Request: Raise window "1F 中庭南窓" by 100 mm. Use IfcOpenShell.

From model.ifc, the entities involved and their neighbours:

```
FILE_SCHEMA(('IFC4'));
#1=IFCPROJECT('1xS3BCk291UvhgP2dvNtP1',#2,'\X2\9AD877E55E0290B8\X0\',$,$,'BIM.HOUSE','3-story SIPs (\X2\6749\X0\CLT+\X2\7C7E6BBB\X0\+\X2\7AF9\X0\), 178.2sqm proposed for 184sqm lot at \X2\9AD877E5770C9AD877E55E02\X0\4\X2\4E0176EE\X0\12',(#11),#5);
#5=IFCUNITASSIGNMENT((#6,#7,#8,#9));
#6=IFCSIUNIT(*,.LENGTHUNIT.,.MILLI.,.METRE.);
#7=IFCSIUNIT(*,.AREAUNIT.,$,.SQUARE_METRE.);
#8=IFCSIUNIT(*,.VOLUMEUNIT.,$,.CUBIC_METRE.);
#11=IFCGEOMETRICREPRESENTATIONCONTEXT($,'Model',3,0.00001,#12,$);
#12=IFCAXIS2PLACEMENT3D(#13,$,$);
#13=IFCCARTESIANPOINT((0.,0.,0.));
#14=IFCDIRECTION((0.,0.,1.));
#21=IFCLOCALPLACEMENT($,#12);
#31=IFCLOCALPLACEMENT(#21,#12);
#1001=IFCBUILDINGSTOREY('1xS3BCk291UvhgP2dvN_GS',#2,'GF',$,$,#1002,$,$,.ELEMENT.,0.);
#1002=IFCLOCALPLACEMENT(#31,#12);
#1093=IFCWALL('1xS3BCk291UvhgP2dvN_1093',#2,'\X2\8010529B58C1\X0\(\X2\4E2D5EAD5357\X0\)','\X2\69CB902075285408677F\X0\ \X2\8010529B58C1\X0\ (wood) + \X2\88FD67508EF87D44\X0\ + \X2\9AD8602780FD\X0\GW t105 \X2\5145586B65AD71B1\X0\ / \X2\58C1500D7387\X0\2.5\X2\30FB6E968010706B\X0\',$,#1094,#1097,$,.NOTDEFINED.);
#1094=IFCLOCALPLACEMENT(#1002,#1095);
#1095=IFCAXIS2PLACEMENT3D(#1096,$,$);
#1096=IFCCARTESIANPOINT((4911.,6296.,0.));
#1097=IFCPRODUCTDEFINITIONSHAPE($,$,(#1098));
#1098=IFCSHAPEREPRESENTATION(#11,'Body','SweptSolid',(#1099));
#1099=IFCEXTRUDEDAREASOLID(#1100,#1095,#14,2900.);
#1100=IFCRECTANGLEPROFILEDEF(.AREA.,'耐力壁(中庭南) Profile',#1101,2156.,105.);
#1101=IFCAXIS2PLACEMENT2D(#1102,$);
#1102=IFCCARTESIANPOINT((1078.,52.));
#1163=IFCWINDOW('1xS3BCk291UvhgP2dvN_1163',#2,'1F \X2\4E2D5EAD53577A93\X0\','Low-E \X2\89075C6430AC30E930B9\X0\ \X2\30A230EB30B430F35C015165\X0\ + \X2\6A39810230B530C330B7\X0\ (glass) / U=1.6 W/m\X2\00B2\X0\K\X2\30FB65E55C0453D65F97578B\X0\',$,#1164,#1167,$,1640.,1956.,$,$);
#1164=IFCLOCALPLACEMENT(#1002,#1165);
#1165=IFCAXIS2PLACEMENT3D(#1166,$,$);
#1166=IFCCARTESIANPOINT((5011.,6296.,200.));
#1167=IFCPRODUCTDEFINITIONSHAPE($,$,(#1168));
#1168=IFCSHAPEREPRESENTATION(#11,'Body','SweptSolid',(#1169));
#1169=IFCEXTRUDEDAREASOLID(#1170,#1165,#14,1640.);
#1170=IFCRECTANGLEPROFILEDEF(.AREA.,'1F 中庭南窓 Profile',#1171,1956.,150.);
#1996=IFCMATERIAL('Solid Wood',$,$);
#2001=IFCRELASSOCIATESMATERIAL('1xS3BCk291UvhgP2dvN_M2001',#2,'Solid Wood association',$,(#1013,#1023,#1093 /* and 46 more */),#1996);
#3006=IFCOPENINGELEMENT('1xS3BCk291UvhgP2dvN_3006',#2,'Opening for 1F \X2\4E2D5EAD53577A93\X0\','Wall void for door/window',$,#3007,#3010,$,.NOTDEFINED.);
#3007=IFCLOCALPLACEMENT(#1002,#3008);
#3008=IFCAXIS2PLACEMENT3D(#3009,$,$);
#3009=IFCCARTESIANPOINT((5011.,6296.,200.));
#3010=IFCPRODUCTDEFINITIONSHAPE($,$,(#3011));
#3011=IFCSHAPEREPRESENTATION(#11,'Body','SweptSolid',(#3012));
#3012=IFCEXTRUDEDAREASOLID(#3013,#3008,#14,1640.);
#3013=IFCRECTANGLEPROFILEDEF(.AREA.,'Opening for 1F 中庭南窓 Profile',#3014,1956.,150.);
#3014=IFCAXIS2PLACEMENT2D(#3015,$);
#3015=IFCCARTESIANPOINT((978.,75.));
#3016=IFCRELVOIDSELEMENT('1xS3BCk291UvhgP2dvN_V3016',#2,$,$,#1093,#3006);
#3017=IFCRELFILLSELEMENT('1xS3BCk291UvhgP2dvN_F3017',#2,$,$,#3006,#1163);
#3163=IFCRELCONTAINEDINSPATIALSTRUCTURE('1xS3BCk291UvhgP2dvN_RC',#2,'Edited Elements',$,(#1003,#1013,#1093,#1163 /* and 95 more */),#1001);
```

```python
import numpy as np
import ifcopenshell
import ifcopenshell.api.geometry
import ifcopenshell.util.placement
import ifcopenshell.util.unit

model = ifcopenshell.open("model.ifc")
unit_scale = ifcopenshell.util.unit.calculate_unit_scale(model)

window = model.by_guid("1xS3BCk291UvhgP2dvN_1163")
opening = window.FillsVoids[0].RelatingOpeningElement
dz = 0.1 / unit_scale

shift = np.array([0.0, 0.0, dz])
# The window is not placed relative to its opening, so move both.
for product in (opening, window):
    matrix = ifcopenshell.util.placement.get_local_placement(product.ObjectPlacement)
    matrix[:3, 3] += shift
    ifcopenshell.api.geometry.edit_object_placement(model, product=product, matrix=matrix, is_si=False)

print(f"moved by {dz * unit_scale:+.3f} m")

model.write("model_rev.ifc")
```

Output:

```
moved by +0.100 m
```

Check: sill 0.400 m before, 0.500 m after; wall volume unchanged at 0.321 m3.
